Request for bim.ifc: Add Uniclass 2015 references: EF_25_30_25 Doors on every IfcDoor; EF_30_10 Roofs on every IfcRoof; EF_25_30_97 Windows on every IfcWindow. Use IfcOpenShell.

First a look at what the model holds.

```python
import ifcopenshell

model = ifcopenshell.open("bim.ifc")
print(model.schema)
print("classifications:", [c.Name for c in model.by_type("IfcClassification")])
for ifc_class in ("IfcDoor", "IfcRoof", "IfcStair", "IfcWall", "IfcWindow"):
    print(ifc_class, len(model.by_type(ifc_class)))
```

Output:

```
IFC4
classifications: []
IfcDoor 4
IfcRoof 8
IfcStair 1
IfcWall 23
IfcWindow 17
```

```python
import ifcopenshell
import ifcopenshell.api.classification

model = ifcopenshell.open("bim.ifc")

system = ifcopenshell.api.classification.add_classification(model, classification="Uniclass 2015")

codes = {
    "IfcDoor": ("EF_25_30_25", "Doors"),
    "IfcRoof": ("EF_30_10", "Roofs"),
    "IfcWindow": ("EF_25_30_97", "Windows"),
}
for ifc_class, (code, name) in codes.items():
    products = model.by_type(ifc_class)
    ifcopenshell.api.classification.add_reference(
        model, products=products, classification=system, identification=code, name=name
    )
    print(code, len(products))

model.write("bim-out.ifc")
```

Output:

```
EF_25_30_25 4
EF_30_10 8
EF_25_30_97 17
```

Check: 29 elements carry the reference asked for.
